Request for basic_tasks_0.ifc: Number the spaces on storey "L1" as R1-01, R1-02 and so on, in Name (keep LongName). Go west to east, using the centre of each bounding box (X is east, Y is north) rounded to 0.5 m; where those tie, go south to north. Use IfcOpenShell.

First a look at what the model holds.

```python
import ifcopenshell
import ifcopenshell.util.element
import ifcopenshell.util.placement

model = ifcopenshell.open("basic_tasks_0.ifc")
print(model.schema)
storey = next(s for s in model.by_type("IfcBuildingStorey") if s.Name == "L1")
spaces = [e for e in ifcopenshell.util.element.get_decomposition(storey) if e.is_a("IfcSpace")]
for e in sorted(spaces, key=lambda e: e.id()):
    origin = ifcopenshell.util.placement.get_local_placement(e.ObjectPlacement)[:3, 3]
    print(e.id(), e.Name, e.LongName, origin.round(2) + 0.0, sep=" | ")
```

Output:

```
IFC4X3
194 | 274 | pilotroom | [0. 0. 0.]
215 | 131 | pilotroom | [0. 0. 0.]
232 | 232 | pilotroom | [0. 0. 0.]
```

```python
import ifcopenshell
import ifcopenshell.geom
import ifcopenshell.util.element
import ifcopenshell.util.shape

model = ifcopenshell.open("basic_tasks_0.ifc")
settings = ifcopenshell.geom.settings()
settings.set("use-world-coords", True)


def centre(element):
    shape = ifcopenshell.geom.create_shape(settings, element)
    return ifcopenshell.util.shape.get_bbox_centroid(shape.geometry)


storey = next(s for s in model.by_type("IfcBuildingStorey") if s.Name == "L1")
spaces = [e for e in ifcopenshell.util.element.get_decomposition(storey) if e.is_a("IfcSpace")]

# Insertion points can sit at a corner or the storey origin, so sort by the geometry (in metres).
centres = {e: centre(e) for e in spaces}
spaces.sort(key=lambda e: (round(centres[e][0] / 0.5), centres[e][1]))

for i, e in enumerate(spaces, start=1):
    number = f"R1-{i:02d}"
    e.Name = number
    print(e.id(), number)

model.write("basic_tasks_0_rev.ifc")
```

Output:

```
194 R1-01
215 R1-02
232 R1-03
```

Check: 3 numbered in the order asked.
